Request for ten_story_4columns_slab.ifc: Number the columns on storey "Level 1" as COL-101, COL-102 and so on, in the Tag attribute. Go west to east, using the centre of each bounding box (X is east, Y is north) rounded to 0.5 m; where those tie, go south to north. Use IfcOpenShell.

First a look at what the model holds.

```python
import ifcopenshell
import ifcopenshell.util.element
import ifcopenshell.util.placement

model = ifcopenshell.open("ten_story_4columns_slab.ifc")
print(model.schema)
storey = next(s for s in model.by_type("IfcBuildingStorey") if s.Name == "Level 1")
columns = [e for e in ifcopenshell.util.element.get_decomposition(storey) if e.is_a("IfcColumn")]
for e in sorted(columns, key=lambda e: e.id()):
    origin = ifcopenshell.util.placement.get_local_placement(e.ObjectPlacement)[:3, 3]
    print(e.id(), e.Tag, e.Name, origin.round(2) + 0.0, sep=" | ")
```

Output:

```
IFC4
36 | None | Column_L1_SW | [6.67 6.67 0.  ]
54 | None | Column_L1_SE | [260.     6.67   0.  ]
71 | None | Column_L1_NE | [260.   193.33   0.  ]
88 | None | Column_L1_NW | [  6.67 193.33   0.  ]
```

```python
import ifcopenshell
import ifcopenshell.geom
import ifcopenshell.util.element
import ifcopenshell.util.shape

model = ifcopenshell.open("ten_story_4columns_slab.ifc")
settings = ifcopenshell.geom.settings()
settings.set("use-world-coords", True)


def centre(element):
    shape = ifcopenshell.geom.create_shape(settings, element)
    return ifcopenshell.util.shape.get_bbox_centroid(shape.geometry)


storey = next(s for s in model.by_type("IfcBuildingStorey") if s.Name == "Level 1")
columns = [e for e in ifcopenshell.util.element.get_decomposition(storey) if e.is_a("IfcColumn")]

# Insertion points can sit at a corner or the storey origin, so sort by the geometry (in metres).
centres = {e: centre(e) for e in columns}
columns.sort(key=lambda e: (round(centres[e][0] / 0.5), centres[e][1]))

for i, e in enumerate(columns, start=1):
    number = f"COL-1{i:02d}"
    e.Tag = number
    print(e.id(), number)

model.write("ten_story_4columns_slab_edited.ifc")
```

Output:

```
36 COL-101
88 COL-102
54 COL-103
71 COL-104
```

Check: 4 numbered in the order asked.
